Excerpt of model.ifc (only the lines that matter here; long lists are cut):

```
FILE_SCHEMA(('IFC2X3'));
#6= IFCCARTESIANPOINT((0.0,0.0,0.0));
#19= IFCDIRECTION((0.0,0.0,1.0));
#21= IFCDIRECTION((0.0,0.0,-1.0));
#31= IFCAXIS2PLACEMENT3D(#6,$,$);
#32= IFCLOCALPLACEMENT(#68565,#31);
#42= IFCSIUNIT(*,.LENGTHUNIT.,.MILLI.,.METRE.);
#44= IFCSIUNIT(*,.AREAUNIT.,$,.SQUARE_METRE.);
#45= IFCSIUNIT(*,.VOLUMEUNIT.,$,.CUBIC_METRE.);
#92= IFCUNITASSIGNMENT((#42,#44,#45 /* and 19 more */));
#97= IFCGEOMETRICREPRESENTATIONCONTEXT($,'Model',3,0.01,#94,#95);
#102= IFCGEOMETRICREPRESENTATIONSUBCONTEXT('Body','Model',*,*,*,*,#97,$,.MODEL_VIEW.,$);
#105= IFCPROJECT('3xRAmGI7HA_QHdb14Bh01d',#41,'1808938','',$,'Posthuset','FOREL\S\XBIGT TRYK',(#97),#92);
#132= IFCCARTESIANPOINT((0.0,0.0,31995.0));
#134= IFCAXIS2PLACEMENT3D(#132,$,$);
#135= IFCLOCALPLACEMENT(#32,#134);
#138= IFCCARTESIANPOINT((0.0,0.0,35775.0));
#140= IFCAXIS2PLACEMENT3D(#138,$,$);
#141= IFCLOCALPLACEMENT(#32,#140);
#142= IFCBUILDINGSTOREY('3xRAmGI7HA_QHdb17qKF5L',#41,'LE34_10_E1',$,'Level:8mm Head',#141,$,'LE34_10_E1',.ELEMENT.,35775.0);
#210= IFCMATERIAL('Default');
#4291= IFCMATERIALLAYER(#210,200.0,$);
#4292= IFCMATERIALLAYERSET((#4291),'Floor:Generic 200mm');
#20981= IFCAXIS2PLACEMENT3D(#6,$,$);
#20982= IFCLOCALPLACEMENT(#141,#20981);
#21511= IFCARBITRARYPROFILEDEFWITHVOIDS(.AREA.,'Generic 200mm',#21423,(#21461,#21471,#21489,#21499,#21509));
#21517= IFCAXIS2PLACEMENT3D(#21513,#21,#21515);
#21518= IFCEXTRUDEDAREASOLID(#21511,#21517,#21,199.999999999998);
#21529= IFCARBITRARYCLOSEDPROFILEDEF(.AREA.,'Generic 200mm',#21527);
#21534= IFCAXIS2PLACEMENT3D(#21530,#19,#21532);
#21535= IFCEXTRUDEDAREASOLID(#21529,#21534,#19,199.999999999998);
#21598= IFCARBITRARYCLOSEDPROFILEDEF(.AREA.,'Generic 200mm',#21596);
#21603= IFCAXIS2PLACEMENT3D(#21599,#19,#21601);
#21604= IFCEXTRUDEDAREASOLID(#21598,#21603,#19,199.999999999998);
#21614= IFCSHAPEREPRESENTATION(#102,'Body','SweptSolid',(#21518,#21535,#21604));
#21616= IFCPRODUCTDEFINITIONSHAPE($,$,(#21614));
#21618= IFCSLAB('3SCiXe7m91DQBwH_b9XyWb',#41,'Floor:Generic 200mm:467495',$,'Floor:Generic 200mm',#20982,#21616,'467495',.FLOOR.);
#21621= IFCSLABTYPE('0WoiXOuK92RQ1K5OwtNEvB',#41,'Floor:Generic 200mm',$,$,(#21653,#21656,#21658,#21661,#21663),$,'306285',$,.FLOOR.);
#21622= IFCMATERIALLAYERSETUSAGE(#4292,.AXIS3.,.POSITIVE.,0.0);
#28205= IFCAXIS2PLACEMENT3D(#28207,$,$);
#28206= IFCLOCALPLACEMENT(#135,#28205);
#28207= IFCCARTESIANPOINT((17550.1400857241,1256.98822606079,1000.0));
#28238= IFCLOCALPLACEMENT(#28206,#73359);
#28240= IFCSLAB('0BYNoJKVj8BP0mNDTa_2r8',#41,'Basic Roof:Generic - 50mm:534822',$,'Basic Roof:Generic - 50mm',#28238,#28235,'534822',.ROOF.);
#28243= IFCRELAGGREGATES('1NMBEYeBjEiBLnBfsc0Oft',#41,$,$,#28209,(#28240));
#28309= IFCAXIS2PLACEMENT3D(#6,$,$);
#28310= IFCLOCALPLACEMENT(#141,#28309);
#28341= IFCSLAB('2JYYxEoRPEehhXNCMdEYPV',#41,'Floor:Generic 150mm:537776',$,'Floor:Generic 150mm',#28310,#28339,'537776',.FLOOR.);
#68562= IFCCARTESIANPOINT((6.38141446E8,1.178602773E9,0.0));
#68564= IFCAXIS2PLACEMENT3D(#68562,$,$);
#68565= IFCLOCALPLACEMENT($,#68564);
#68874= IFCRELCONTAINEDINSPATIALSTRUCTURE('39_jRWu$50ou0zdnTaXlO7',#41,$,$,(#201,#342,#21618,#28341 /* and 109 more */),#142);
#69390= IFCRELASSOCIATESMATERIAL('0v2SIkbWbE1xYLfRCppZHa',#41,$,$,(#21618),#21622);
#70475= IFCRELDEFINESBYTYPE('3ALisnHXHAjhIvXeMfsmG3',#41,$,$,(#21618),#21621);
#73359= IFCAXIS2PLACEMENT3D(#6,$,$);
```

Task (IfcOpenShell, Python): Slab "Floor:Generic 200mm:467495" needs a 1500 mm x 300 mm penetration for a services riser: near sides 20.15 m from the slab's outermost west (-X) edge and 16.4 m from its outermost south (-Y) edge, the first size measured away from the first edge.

```python
import numpy as np
import ifcopenshell
import ifcopenshell.api.feature
import ifcopenshell.api.geometry
import ifcopenshell.api.root
import ifcopenshell.geom
import ifcopenshell.util.placement
import ifcopenshell.util.representation
import ifcopenshell.util.shape
import ifcopenshell.util.unit

model = ifcopenshell.open("model.ifc")
unit_scale = ifcopenshell.util.unit.calculate_unit_scale(model)
settings = ifcopenshell.geom.settings()


def volume(element):
    """Net volume in cubic metres, openings subtracted."""
    shape = ifcopenshell.geom.create_shape(settings, element)
    return ifcopenshell.util.shape.get_volume(shape.geometry)


slab = model.by_guid("3SCiXe7m91DQBwH_b9XyWb")
before = volume(slab)

# Extent in the slab's own axes, in metres. The edges named are its -X and -Y sides.
slab_shape = ifcopenshell.geom.create_shape(settings, slab)
vertices = ifcopenshell.util.shape.get_vertices(slab_shape.geometry)
x_min, y_min, bottom = vertices.min(axis=0)
top = vertices[:, 2].max()

opening = ifcopenshell.api.root.create_entity(model, ifc_class="IfcOpeningElement", name="Services riser opening")
context = ifcopenshell.util.representation.get_context(model, "Model", "Body", "MODEL_VIEW")
width, depth = 1.5, 0.3
outline = [(0.0, 0.0), (width, 0.0), (width, depth), (0.0, depth), (0.0, 0.0)]
# Overshoot both faces by 50 mm so the cut is clean.
shape = ifcopenshell.api.geometry.add_slab_representation(
    model, context=context, depth=top - bottom + 0.1, polyline=outline
)
ifcopenshell.api.geometry.assign_representation(model, product=opening, representation=shape)

matrix = ifcopenshell.util.placement.get_local_placement(slab.ObjectPlacement)
matrix[:, 3] = matrix @ np.append(np.array([x_min + 20.15, y_min + 16.4, bottom - 0.05]) / unit_scale, 1.0)
ifcopenshell.api.geometry.edit_object_placement(model, product=opening, matrix=matrix, is_si=False)
ifcopenshell.api.feature.add_feature(model, feature=opening, element=slab)

after = volume(slab)

print(f"slab volume {before:.3f} -> {after:.3f} m3")

model.write("model-out.ifc")
```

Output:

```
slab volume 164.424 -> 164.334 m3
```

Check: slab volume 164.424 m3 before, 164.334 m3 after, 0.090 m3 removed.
